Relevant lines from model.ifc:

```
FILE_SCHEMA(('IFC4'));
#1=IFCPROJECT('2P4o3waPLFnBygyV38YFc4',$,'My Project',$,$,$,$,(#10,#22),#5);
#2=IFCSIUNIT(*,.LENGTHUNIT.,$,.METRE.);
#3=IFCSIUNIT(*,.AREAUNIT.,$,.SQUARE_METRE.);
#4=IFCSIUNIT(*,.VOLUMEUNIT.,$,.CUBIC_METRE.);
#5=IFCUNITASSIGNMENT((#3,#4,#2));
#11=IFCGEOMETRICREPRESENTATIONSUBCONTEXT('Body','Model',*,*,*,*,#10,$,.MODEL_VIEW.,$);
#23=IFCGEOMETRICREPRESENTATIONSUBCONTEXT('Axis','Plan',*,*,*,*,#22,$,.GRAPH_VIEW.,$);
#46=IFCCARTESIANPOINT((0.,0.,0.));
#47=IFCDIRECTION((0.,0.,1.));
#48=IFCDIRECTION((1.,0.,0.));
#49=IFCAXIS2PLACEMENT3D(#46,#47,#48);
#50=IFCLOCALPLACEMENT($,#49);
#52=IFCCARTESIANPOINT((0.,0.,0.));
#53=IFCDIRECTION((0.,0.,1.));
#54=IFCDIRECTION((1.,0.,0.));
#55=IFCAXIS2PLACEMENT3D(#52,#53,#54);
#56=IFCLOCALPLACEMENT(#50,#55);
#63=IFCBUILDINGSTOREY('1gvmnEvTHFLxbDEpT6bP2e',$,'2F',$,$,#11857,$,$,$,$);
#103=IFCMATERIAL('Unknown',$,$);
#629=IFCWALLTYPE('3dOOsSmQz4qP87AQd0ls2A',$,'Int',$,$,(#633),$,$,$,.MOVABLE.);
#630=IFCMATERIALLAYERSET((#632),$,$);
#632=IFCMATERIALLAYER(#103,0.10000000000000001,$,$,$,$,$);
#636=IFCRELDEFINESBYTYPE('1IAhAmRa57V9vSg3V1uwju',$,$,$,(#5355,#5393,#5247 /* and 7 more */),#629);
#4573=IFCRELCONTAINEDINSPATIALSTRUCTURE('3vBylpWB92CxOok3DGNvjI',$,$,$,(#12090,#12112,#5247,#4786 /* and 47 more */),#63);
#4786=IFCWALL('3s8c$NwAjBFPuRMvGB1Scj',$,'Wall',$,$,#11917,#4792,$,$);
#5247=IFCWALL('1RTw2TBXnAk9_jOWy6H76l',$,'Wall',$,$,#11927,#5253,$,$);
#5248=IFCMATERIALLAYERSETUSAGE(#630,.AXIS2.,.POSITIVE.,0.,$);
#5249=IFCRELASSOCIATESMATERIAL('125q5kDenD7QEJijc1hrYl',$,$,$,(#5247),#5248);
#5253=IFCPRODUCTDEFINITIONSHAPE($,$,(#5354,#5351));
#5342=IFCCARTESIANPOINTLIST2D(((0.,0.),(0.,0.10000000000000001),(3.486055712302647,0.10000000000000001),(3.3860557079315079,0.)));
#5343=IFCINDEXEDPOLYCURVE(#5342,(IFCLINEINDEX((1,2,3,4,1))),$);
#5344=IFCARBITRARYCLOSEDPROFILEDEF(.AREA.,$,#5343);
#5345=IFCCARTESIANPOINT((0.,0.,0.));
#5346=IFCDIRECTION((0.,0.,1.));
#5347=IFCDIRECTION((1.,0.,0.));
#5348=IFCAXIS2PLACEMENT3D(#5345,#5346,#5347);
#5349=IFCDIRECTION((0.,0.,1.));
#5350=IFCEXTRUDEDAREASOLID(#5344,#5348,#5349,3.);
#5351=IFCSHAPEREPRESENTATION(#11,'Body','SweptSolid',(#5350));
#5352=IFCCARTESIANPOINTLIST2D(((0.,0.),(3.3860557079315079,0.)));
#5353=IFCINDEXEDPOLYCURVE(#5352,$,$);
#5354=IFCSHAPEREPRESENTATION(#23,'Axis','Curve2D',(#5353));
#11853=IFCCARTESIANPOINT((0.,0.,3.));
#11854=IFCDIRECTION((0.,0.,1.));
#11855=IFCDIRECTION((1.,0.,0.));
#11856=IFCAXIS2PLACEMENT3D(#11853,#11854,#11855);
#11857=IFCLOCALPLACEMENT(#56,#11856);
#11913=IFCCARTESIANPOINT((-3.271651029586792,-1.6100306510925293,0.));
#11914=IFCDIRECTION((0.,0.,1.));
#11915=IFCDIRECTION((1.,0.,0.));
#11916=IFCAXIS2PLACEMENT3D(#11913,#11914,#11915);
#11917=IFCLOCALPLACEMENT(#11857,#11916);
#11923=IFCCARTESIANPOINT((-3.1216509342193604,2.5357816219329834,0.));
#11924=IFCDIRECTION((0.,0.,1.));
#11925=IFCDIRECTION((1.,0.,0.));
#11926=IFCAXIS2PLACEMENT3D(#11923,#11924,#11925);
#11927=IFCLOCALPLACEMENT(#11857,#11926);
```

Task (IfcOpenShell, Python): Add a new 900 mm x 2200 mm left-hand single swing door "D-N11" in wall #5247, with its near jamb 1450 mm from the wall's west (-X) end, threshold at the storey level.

```python
import numpy as np
import ifcopenshell
import ifcopenshell.api.feature
import ifcopenshell.api.geometry
import ifcopenshell.api.root
import ifcopenshell.api.spatial
import ifcopenshell.geom
import ifcopenshell.util.element
import ifcopenshell.util.placement
import ifcopenshell.util.representation
import ifcopenshell.util.shape
import ifcopenshell.util.unit

model = ifcopenshell.open("model.ifc")
unit_scale = ifcopenshell.util.unit.calculate_unit_scale(model)
settings = ifcopenshell.geom.settings()


def volume(element):
    """Net volume in cubic metres, openings subtracted."""
    shape = ifcopenshell.geom.create_shape(settings, element)
    return ifcopenshell.util.shape.get_volume(shape.geometry)


wall = model.by_guid("1RTw2TBXnAk9_jOWy6H76l")
storey = ifcopenshell.util.element.get_container(wall, ifc_class="IfcBuildingStorey")
context = ifcopenshell.util.representation.get_context(model, "Model", "Body", "MODEL_VIEW")
before = volume(wall)

width, height, from_end, sill = 0.9, 2.2, 1.45, 0.0  # metres

# The wall runs along its own X axis, and the end named is its -X end.
wall_shape = ifcopenshell.geom.create_shape(settings, wall)
x, y, z = ifcopenshell.util.shape.get_vertices(wall_shape.geometry).T
start = x.min() + from_end
face, thickness = float(y.min()), float(y.max() - y.min())
wall_matrix = ifcopenshell.util.placement.get_local_placement(wall.ObjectPlacement)
level = ifcopenshell.util.placement.get_local_placement(storey.ObjectPlacement)[2, 3]


def in_wall(x, y):
    """Placement at x, y metres in the wall's axes, at sill height."""
    matrix = wall_matrix.copy()
    matrix[:, 3] = wall_matrix @ np.array([x / unit_scale, y / unit_scale, 0.0, 1.0])
    matrix[2, 3] = level + sill / unit_scale
    return matrix


# Opening: a box that overshoots both wall faces by 50 mm.
opening = ifcopenshell.api.root.create_entity(model, ifc_class="IfcOpeningElement", predefined_type="OPENING")
box = ifcopenshell.api.geometry.add_wall_representation(
    model, context=context, length=width, height=height, thickness=thickness + 0.1
)
ifcopenshell.api.geometry.assign_representation(model, product=opening, representation=box)
ifcopenshell.api.geometry.edit_object_placement(model, product=opening, matrix=in_wall(start, face - 0.05), is_si=False)
ifcopenshell.api.feature.add_feature(model, feature=opening, element=wall)

door = ifcopenshell.api.root.create_entity(model, ifc_class="IfcDoor", name="D-N11", predefined_type="DOOR")
door.OverallWidth, door.OverallHeight = width / unit_scale, height / unit_scale
door.OperationType = "SINGLE_SWING_LEFT"
body = ifcopenshell.api.geometry.add_door_representation(
    model,
    context=context,
    overall_width=door.OverallWidth,
    overall_height=door.OverallHeight,
    operation_type="SINGLE_SWING_LEFT",
    lining_properties={"LiningDepth": thickness / unit_scale, "ThresholdDepth": thickness / unit_scale},
)
ifcopenshell.api.geometry.assign_representation(model, product=door, representation=body)
ifcopenshell.api.spatial.assign_container(model, products=[door], relating_structure=storey)
ifcopenshell.api.feature.add_filling(model, opening=opening, element=door)

# The lining spans the wall, so the door starts at the wall face.
ifcopenshell.api.geometry.edit_object_placement(model, product=door, matrix=in_wall(start, face), is_si=False)

after = volume(wall)

print(f"wall volume {before:.3f} -> {after:.3f} m3")

model.write("model_updated.ifc")
```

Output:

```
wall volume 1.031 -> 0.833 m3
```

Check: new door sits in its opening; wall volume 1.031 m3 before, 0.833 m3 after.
